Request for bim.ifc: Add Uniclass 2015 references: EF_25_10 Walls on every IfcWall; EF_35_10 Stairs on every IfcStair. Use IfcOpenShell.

First a look at what the model holds.

```python
import ifcopenshell

model = ifcopenshell.open("bim.ifc")
print(model.schema)
print("classifications:", [c.Name for c in model.by_type("IfcClassification")])
for ifc_class in ("IfcDoor", "IfcRoof", "IfcStair", "IfcWall", "IfcWindow"):
    print(ifc_class, len(model.by_type(ifc_class)))
```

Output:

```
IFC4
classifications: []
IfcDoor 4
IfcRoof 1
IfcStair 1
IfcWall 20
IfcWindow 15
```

```python
import ifcopenshell
import ifcopenshell.api.classification

model = ifcopenshell.open("bim.ifc")

system = ifcopenshell.api.classification.add_classification(model, classification="Uniclass 2015")

codes = {
    "IfcWall": ("EF_25_10", "Walls"),
    "IfcStair": ("EF_35_10", "Stairs"),
}
for ifc_class, (code, name) in codes.items():
    products = model.by_type(ifc_class)
    ifcopenshell.api.classification.add_reference(
        model, products=products, classification=system, identification=code, name=name
    )
    print(code, len(products))

model.write("bim_rev.ifc")
```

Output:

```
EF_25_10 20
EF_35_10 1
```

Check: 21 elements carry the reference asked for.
